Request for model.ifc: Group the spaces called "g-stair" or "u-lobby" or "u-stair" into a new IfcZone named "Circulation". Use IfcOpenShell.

First a look at what the model holds.

```python
import ifcopenshell

model = ifcopenshell.open("model.ifc")
print(model.schema)
seen = {}
for space in model.by_type("IfcSpace"):
    seen[space.LongName] = seen.get(space.LongName, 0) + 1
for name, count in sorted(seen.items(), key=str):
    print(count, "x", name)
print("zones:", [z.Name for z in model.by_type("IfcZone")][:20])
```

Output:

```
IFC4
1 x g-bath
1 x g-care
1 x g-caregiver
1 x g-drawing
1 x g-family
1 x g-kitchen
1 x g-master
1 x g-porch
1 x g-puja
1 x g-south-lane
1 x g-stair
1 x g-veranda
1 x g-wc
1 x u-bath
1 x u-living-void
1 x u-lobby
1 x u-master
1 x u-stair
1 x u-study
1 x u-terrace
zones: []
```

```python
import ifcopenshell
import ifcopenshell.api.group
import ifcopenshell.api.root

model = ifcopenshell.open("model.ifc")

names = {"g-stair", "u-lobby", "u-stair"}
spaces = [s for s in model.by_type("IfcSpace") if s.LongName in names]

zone = ifcopenshell.api.root.create_entity(model, ifc_class="IfcZone", name="Circulation")
ifcopenshell.api.group.assign_group(model, products=spaces, group=zone)
print(len(spaces), "spaces in", zone.Name)

model.write("model_v2.ifc")
```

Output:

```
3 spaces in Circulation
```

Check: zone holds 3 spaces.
